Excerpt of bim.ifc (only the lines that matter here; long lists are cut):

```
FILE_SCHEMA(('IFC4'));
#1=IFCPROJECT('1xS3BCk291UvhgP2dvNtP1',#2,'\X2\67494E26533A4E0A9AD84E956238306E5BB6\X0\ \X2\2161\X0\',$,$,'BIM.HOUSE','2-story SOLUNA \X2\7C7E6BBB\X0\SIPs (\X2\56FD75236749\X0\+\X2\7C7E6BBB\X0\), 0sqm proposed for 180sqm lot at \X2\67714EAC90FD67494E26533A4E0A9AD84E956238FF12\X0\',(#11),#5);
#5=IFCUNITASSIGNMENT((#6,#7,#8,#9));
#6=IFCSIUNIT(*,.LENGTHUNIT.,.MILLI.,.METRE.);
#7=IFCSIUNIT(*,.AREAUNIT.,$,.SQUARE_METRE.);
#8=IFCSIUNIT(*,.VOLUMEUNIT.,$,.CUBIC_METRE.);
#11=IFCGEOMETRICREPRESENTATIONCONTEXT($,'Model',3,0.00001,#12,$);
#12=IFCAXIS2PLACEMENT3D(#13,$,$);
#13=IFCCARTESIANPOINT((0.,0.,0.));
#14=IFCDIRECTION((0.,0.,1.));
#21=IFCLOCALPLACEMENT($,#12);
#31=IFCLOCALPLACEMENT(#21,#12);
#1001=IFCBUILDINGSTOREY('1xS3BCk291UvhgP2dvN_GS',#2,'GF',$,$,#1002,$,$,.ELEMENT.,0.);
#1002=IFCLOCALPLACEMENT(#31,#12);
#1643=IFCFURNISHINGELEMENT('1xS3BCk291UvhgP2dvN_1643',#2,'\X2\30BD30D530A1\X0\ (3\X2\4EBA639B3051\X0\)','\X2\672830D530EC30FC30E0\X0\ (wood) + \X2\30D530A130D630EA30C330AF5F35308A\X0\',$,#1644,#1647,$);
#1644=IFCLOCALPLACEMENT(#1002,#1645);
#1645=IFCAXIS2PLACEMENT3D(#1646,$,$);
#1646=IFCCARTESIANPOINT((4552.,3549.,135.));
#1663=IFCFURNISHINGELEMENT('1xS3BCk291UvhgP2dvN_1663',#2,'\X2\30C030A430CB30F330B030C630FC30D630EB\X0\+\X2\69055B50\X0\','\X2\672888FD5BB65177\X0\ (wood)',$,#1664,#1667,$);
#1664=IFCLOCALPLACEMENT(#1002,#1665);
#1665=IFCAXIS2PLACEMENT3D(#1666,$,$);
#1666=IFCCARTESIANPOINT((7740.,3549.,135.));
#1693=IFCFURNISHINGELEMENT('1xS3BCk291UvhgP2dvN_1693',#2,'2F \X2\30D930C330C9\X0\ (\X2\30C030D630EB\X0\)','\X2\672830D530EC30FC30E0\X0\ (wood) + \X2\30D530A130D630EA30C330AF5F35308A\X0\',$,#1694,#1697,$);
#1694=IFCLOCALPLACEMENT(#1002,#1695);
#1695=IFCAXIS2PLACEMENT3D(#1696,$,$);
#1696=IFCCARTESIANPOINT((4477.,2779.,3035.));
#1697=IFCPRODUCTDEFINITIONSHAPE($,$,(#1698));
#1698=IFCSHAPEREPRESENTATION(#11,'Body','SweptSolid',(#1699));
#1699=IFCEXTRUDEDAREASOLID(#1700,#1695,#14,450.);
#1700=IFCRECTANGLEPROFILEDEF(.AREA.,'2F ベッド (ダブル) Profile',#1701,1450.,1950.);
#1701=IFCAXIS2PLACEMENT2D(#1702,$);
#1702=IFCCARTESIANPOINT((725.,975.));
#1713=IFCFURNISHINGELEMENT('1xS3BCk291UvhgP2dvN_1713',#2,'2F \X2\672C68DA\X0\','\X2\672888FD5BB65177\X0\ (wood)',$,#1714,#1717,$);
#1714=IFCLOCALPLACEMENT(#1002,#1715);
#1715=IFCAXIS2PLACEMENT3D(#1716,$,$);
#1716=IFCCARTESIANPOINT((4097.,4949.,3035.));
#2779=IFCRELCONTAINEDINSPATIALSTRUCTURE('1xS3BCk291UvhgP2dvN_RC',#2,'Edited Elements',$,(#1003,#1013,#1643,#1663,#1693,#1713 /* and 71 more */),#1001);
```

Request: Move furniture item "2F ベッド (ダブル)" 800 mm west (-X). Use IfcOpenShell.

```python
import ifcopenshell
import ifcopenshell.api.geometry
import ifcopenshell.util.placement

model = ifcopenshell.open("bim.ifc")

item = model.by_guid("1xS3BCk291UvhgP2dvN_1693")
matrix = ifcopenshell.util.placement.get_local_placement(item.ObjectPlacement)
matrix[0, 3] -= 800.0
ifcopenshell.api.geometry.edit_object_placement(model, product=item, matrix=matrix, is_si=False)

print(ifcopenshell.util.placement.get_local_placement(item.ObjectPlacement).round(3) + 0.0)

model.write("bim_rev.ifc")
```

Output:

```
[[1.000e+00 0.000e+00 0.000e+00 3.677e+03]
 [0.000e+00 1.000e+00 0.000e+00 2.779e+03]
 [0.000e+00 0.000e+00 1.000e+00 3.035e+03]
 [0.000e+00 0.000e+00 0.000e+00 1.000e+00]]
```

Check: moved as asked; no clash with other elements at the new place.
